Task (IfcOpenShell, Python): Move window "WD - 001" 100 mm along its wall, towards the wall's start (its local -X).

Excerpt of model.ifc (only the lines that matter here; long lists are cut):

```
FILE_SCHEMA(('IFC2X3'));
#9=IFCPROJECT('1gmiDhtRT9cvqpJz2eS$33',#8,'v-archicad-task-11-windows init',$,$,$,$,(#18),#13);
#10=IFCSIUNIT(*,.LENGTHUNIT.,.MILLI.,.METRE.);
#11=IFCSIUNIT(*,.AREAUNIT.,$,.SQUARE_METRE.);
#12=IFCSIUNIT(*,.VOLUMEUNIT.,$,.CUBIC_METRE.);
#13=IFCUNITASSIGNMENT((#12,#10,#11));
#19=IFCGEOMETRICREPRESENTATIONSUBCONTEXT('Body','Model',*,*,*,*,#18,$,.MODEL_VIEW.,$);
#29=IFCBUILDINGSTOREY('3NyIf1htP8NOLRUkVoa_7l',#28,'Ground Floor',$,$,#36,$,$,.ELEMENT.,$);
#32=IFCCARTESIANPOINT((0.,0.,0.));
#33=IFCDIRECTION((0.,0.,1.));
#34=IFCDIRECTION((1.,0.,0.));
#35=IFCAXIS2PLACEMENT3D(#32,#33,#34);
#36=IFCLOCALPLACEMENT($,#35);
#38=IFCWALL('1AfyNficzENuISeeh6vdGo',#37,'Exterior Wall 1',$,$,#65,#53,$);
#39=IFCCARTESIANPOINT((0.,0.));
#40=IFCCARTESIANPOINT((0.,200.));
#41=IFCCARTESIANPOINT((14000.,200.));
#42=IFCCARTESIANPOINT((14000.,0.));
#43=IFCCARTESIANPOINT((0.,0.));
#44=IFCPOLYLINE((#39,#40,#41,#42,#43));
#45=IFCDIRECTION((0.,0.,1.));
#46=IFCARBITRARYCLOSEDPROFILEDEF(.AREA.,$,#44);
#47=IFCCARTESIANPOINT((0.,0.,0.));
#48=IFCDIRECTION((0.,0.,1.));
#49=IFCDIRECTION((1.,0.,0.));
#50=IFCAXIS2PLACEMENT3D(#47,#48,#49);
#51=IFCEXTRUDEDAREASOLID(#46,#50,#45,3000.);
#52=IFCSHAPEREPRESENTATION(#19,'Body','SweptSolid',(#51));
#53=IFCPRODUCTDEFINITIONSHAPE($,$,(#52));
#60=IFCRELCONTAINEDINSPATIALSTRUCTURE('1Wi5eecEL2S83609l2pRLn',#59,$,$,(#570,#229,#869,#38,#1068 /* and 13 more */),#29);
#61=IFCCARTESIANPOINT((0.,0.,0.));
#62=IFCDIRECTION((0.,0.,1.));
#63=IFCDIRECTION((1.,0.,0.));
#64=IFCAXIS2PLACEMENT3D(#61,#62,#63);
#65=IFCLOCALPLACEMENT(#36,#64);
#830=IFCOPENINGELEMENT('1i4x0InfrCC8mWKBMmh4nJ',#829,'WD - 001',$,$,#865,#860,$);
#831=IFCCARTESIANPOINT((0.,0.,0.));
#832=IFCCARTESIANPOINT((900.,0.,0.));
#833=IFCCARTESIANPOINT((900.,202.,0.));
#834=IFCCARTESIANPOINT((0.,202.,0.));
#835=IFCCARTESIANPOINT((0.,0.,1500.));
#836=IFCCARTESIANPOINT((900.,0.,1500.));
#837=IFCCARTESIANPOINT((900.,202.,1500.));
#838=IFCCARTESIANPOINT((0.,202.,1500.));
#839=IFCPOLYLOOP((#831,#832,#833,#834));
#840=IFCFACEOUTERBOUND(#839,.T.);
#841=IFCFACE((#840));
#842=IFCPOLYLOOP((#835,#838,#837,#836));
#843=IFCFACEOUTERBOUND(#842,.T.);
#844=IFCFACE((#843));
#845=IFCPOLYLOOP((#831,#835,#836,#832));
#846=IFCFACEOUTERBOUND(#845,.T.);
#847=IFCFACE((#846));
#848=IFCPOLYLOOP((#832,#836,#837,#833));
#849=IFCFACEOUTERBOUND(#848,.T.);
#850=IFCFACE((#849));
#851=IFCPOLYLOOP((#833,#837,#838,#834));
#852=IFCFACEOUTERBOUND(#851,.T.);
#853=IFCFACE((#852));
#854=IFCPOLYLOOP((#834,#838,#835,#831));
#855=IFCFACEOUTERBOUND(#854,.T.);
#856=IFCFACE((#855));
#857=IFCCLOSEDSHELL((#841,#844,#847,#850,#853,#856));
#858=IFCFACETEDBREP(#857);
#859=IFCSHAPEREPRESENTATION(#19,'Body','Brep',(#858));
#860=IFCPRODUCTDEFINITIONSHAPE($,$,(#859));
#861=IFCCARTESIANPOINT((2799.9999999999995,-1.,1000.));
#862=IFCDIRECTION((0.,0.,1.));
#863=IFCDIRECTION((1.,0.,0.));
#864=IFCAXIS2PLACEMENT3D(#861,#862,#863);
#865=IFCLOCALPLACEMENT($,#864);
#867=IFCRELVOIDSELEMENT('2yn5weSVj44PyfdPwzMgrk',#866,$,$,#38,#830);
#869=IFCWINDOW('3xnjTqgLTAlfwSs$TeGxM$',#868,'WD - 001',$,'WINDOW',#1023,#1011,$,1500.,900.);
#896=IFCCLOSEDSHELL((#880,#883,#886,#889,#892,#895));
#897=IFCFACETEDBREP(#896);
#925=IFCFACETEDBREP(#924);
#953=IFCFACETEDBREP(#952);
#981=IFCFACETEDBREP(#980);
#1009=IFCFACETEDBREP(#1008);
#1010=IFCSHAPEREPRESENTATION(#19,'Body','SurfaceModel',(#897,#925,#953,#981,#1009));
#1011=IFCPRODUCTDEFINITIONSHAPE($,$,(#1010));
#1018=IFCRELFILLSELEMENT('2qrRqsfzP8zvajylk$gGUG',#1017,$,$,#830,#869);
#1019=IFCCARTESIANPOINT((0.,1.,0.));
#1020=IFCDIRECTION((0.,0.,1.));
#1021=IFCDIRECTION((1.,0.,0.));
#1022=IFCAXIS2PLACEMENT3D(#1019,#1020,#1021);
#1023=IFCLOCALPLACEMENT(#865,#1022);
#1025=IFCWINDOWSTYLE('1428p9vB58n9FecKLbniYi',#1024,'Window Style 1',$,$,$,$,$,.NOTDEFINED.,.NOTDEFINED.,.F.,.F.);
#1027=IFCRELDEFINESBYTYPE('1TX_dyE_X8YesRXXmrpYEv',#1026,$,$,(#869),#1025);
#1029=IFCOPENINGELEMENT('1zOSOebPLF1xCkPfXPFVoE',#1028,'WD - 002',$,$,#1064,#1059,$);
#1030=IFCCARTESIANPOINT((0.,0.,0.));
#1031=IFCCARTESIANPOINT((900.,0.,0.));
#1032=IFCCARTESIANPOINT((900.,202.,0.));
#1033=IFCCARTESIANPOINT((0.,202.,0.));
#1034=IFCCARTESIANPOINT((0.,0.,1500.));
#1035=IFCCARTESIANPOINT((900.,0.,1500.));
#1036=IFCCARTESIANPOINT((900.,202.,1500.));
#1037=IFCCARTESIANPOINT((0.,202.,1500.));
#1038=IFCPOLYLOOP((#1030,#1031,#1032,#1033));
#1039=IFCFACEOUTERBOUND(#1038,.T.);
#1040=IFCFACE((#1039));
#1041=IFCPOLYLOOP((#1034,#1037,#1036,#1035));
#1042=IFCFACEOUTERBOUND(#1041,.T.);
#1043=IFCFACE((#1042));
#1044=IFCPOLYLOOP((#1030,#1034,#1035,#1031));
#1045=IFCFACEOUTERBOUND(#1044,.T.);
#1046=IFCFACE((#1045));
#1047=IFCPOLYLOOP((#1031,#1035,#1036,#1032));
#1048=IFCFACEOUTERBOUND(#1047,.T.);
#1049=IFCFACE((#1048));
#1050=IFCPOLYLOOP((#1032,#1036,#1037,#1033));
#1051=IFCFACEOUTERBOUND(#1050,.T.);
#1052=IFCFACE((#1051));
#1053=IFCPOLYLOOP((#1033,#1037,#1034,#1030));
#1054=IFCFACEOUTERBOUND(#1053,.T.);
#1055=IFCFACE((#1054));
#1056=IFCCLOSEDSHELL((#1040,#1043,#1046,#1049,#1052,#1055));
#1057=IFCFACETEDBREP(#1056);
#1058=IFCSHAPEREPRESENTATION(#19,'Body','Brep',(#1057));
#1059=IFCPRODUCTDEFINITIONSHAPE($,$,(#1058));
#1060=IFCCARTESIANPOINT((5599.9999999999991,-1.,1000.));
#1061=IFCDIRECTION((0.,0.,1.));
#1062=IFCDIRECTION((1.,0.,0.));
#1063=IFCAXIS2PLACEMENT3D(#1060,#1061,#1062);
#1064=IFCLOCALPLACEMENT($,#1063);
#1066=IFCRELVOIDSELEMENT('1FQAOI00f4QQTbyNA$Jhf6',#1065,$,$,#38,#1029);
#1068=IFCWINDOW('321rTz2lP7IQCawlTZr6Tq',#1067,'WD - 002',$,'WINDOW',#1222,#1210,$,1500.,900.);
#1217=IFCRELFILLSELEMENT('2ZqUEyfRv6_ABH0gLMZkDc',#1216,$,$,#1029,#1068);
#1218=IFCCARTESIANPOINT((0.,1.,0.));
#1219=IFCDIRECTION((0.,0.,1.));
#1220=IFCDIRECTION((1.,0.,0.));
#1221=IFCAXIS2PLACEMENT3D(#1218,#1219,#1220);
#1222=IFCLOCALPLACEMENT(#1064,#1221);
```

```python
import ifcopenshell
import ifcopenshell.api.geometry
import ifcopenshell.util.placement

model = ifcopenshell.open("model.ifc")

window = model.by_guid("3xnjTqgLTAlfwSs$TeGxM$")
opening = window.FillsVoids[0].RelatingOpeningElement
wall = opening.VoidsElements[0].RelatingBuildingElement

wall_matrix = ifcopenshell.util.placement.get_local_placement(wall.ObjectPlacement)
shift = wall_matrix[:3, 0] * -100.0
before = ifcopenshell.util.placement.get_local_placement(window.ObjectPlacement)[:3, 3].copy()

# The window is placed relative to its opening, so it follows when the opening moves.
matrix = ifcopenshell.util.placement.get_local_placement(opening.ObjectPlacement)
matrix[:3, 3] += shift
ifcopenshell.api.geometry.edit_object_placement(
    model, product=opening, matrix=matrix, is_si=False, should_transform_children=True
)

after = ifcopenshell.util.placement.get_local_placement(window.ObjectPlacement)[:3, 3]
print("window moved by", (after - before).round(3) + 0.0)

model.write("model_edited.ifc")
```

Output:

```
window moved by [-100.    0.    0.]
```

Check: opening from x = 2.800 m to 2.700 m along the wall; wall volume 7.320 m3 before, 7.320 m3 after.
